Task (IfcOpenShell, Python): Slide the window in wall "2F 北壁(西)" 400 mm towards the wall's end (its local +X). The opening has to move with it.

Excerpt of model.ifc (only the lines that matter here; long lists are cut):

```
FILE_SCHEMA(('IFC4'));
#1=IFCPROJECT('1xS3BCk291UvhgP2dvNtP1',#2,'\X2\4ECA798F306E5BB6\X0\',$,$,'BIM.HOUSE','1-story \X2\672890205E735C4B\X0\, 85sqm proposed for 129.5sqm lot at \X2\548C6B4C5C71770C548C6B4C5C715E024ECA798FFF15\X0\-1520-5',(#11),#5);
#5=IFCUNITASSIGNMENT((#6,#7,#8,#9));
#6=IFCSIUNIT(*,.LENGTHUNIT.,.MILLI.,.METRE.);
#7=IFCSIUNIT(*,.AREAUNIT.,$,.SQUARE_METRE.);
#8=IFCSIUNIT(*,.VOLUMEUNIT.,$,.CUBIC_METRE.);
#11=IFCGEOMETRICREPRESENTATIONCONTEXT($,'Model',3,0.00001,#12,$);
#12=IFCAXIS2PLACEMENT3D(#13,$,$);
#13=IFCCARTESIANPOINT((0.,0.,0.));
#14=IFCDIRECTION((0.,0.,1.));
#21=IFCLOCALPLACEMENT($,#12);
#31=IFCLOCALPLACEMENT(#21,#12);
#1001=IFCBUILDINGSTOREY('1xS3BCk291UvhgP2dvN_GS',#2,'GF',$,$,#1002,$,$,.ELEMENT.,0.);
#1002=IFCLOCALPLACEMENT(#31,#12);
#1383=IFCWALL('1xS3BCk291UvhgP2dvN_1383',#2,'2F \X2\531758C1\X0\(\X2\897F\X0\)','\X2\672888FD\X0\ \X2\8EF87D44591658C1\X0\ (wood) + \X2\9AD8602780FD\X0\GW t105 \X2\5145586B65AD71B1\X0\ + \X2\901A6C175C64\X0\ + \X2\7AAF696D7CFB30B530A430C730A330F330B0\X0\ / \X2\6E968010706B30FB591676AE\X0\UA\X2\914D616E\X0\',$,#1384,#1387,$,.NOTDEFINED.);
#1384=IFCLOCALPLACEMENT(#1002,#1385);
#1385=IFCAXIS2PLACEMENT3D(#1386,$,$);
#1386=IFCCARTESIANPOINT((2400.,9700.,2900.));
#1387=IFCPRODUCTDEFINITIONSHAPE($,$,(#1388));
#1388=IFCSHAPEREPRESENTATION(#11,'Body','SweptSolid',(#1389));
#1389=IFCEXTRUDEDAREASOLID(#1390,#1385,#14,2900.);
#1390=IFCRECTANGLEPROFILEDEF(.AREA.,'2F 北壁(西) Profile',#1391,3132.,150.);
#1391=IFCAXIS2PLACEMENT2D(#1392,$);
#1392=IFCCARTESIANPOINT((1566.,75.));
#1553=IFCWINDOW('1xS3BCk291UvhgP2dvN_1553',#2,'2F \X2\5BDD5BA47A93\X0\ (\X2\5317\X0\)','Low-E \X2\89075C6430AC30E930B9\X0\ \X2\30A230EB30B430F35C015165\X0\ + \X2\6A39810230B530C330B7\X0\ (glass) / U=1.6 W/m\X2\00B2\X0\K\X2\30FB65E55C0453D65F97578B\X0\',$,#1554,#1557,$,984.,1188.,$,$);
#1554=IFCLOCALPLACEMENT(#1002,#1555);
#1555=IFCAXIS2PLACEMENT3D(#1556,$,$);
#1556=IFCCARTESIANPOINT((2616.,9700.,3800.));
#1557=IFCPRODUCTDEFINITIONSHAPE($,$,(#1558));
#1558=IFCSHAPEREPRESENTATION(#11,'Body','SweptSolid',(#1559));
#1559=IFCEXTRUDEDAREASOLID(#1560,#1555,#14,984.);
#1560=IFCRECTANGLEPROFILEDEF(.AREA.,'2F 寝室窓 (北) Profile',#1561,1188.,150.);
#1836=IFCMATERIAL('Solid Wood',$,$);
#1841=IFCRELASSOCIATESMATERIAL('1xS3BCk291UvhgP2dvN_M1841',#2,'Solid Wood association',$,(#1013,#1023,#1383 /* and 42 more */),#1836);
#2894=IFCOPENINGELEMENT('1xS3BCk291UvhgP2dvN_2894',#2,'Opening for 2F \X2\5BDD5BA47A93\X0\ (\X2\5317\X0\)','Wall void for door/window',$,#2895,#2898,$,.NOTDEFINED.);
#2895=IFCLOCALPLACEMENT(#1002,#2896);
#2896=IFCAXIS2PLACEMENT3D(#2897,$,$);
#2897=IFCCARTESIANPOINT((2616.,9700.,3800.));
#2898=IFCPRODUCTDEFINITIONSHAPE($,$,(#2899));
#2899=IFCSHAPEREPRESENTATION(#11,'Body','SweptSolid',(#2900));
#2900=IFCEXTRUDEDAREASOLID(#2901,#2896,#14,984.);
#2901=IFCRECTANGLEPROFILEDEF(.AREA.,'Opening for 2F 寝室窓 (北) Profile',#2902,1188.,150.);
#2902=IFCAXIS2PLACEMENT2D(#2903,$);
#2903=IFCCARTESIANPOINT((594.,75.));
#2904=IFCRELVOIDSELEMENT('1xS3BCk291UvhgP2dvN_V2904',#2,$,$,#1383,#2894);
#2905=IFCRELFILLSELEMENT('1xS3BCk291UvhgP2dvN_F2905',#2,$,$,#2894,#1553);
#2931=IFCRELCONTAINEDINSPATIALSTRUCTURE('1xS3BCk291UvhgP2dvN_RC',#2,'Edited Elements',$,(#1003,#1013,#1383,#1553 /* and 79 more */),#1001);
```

```python
import ifcopenshell
import ifcopenshell.api.geometry
import ifcopenshell.util.placement
import ifcopenshell.util.unit

model = ifcopenshell.open("model.ifc")
unit_scale = ifcopenshell.util.unit.calculate_unit_scale(model)

window = model.by_id(1553)
opening = window.FillsVoids[0].RelatingOpeningElement
wall = opening.VoidsElements[0].RelatingBuildingElement

wall_matrix = ifcopenshell.util.placement.get_local_placement(wall.ObjectPlacement)
shift = wall_matrix[:3, 0] * 0.4 / unit_scale
before = ifcopenshell.util.placement.get_local_placement(window.ObjectPlacement)[:3, 3].copy()

# The window is not placed relative to its opening, so move both.
for product in (opening, window):
    matrix = ifcopenshell.util.placement.get_local_placement(product.ObjectPlacement)
    matrix[:3, 3] += shift
    ifcopenshell.api.geometry.edit_object_placement(model, product=product, matrix=matrix, is_si=False)

after = ifcopenshell.util.placement.get_local_placement(window.ObjectPlacement)[:3, 3]
print("window moved by", (after - before).round(3) + 0.0)

model.write("model_updated.ifc")
```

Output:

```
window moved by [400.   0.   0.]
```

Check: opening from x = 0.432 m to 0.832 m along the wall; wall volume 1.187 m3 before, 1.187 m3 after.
